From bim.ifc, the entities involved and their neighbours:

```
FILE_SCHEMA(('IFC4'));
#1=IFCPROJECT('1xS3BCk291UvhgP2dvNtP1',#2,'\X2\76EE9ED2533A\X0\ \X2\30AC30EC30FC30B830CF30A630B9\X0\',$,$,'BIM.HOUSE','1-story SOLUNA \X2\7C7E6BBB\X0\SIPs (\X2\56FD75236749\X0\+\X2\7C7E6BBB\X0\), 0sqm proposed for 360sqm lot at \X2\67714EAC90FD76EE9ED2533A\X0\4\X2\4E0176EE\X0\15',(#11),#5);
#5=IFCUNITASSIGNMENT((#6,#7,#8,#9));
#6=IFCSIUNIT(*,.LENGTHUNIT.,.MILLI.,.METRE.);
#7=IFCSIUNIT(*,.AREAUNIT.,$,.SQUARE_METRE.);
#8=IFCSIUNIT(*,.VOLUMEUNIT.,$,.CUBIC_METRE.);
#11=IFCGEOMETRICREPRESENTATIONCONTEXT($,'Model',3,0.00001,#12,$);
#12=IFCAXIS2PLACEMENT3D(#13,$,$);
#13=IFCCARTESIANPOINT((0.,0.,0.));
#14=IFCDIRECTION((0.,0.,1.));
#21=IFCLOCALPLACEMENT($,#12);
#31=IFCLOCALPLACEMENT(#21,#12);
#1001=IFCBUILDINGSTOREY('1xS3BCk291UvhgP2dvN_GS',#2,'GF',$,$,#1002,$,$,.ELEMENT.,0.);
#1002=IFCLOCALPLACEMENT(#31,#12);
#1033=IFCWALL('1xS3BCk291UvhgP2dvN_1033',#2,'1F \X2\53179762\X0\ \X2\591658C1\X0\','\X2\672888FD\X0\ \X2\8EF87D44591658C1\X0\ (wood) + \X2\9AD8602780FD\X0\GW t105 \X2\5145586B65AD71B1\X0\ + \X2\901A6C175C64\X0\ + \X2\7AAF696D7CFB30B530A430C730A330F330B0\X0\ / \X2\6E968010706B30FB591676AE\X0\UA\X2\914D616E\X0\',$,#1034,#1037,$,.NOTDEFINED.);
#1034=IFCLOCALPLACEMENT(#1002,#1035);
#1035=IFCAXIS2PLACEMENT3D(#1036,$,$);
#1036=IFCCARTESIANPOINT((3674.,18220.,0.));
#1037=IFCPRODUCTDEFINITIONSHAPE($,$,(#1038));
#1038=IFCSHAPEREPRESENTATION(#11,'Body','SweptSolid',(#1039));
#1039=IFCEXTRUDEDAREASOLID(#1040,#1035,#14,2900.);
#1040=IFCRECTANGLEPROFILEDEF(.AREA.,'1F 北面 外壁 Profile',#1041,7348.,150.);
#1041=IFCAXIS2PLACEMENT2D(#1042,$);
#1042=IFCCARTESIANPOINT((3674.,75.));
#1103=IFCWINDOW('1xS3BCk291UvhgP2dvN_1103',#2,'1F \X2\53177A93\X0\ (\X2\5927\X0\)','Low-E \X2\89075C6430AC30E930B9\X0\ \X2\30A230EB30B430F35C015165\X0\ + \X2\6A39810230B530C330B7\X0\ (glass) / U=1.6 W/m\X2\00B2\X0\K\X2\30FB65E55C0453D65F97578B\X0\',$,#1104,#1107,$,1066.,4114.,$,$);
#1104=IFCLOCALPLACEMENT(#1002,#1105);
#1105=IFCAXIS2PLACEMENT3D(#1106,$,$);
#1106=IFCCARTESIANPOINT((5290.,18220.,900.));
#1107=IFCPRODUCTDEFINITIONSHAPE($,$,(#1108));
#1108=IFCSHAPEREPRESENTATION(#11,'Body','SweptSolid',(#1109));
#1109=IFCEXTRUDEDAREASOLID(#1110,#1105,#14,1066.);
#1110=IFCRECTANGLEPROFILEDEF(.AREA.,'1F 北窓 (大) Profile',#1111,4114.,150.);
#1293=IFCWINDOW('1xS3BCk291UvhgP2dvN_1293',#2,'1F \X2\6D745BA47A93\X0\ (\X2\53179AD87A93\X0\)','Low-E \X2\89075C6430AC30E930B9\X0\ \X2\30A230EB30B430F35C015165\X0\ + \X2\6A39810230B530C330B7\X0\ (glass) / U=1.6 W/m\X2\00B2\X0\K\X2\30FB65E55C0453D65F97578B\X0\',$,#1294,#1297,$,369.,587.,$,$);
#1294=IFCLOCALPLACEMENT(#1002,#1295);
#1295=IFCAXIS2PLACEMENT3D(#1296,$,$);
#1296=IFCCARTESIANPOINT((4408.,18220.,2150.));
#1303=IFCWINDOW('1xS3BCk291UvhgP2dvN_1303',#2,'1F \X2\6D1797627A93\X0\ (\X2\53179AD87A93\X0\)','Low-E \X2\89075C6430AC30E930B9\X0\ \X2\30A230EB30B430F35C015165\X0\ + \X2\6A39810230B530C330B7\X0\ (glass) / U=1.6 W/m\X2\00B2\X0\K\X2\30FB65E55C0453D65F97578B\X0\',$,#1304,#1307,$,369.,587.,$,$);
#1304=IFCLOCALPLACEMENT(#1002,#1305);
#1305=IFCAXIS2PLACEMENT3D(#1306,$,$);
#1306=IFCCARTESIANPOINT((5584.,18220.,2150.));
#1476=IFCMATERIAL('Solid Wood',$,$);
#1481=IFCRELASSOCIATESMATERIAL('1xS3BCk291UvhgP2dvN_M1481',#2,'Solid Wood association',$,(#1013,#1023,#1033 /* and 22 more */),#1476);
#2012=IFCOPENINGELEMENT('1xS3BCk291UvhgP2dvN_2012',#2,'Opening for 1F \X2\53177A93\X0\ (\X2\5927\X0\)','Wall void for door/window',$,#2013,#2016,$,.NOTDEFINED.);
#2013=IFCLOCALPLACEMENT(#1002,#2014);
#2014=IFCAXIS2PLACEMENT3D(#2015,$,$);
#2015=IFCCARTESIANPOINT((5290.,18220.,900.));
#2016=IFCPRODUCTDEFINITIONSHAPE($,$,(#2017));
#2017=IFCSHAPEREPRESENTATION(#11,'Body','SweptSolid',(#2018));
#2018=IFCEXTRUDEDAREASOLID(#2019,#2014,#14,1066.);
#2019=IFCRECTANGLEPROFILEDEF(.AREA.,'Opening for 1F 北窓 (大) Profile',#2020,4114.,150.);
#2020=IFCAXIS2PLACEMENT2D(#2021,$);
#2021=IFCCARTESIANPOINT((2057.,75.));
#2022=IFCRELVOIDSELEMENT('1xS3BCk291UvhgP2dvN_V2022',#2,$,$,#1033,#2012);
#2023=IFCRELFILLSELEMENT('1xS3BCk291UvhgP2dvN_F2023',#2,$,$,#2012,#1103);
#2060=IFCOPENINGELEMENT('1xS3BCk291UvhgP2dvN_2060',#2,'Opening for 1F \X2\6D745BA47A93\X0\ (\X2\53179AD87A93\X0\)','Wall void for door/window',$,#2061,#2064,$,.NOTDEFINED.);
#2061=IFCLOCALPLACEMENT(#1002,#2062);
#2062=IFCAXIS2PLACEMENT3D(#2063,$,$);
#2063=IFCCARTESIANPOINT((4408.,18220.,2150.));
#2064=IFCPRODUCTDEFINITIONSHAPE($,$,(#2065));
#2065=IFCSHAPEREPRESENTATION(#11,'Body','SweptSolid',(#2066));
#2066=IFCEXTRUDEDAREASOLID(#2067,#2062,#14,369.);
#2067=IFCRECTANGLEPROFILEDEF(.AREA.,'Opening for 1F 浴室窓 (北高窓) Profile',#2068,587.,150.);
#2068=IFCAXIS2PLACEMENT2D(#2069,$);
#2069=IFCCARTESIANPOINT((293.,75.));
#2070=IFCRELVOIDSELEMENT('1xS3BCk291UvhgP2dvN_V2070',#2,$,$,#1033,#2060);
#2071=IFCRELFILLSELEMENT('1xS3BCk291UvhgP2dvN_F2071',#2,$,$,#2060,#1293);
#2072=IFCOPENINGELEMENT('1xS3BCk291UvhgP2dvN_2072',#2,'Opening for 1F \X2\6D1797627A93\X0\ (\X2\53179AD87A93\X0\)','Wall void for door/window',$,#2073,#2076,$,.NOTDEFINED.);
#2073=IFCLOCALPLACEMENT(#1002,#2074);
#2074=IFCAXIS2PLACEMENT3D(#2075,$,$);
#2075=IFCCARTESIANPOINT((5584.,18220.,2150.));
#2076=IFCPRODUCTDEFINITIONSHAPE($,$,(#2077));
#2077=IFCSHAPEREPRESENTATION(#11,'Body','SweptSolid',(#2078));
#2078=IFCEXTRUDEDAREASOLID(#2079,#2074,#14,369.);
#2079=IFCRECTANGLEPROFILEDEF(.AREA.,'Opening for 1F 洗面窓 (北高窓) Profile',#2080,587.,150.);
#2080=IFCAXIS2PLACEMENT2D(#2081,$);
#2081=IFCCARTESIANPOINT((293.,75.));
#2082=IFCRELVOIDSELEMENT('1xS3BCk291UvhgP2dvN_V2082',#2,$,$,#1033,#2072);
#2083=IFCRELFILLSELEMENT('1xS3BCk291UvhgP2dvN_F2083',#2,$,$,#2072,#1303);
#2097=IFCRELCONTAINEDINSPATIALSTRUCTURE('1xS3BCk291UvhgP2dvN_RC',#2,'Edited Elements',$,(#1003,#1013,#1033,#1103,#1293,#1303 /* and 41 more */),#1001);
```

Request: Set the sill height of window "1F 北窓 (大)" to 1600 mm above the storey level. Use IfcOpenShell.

```python
import numpy as np
import ifcopenshell
import ifcopenshell.api.geometry
import ifcopenshell.geom
import ifcopenshell.util.element
import ifcopenshell.util.placement
import ifcopenshell.util.shape
import ifcopenshell.util.unit

model = ifcopenshell.open("bim.ifc")
unit_scale = ifcopenshell.util.unit.calculate_unit_scale(model)

window = model.by_guid("1xS3BCk291UvhgP2dvN_1103")
opening = window.FillsVoids[0].RelatingOpeningElement
storey = ifcopenshell.util.element.get_container(window, ifc_class="IfcBuildingStorey")
level = ifcopenshell.util.placement.get_local_placement(storey.ObjectPlacement)[2, 3]

# The opening's origin need not be at the sill, so measure its lowest point.
shape = ifcopenshell.geom.create_shape(ifcopenshell.geom.settings(), opening)
bottom = ifcopenshell.util.shape.get_shape_bottom_elevation(shape, shape.geometry) / unit_scale
dz = level + 1.6 / unit_scale - bottom

shift = np.array([0.0, 0.0, dz])
# The window is not placed relative to its opening, so move both.
for product in (opening, window):
    matrix = ifcopenshell.util.placement.get_local_placement(product.ObjectPlacement)
    matrix[:3, 3] += shift
    ifcopenshell.api.geometry.edit_object_placement(model, product=product, matrix=matrix, is_si=False)

print(f"moved by {dz * unit_scale:+.3f} m")

model.write("bim_edited.ifc")
```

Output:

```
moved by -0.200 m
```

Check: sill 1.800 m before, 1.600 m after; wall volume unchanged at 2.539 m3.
